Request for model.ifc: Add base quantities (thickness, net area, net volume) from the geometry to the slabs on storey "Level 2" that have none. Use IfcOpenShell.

First a look at what the model holds.

```python
import ifcopenshell
import ifcopenshell.util.element
import ifcopenshell.util.unit

model = ifcopenshell.open("model.ifc")
print(model.schema)
for unit_type in ("LENGTHUNIT", "AREAUNIT", "VOLUMEUNIT"):
    print(unit_type, ifcopenshell.util.unit.calculate_unit_scale(model, unit_type))
storey = next(s for s in model.by_type("IfcBuildingStorey") if s.Name == "Level 2")
slabs = [e for e in ifcopenshell.util.element.get_decomposition(storey) if e.is_a("IfcSlab")]
for e in sorted(slabs, key=lambda e: e.id()):
    print(e.id(), e.is_a(), e.Name, list(ifcopenshell.util.element.get_psets(e, qtos_only=True)), sep=" | ")
```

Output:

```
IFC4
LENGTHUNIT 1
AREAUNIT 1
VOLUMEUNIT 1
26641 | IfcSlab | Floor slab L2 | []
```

```python
import ifcopenshell
import ifcopenshell.api.pset
import ifcopenshell.geom
import ifcopenshell.util.element
import ifcopenshell.util.shape
import ifcopenshell.util.unit

model = ifcopenshell.open("model.ifc")
unit_scale = ifcopenshell.util.unit.calculate_unit_scale(model)
area_scale = ifcopenshell.util.unit.calculate_unit_scale(model, "AREAUNIT")
volume_scale = ifcopenshell.util.unit.calculate_unit_scale(model, "VOLUMEUNIT")
settings = ifcopenshell.geom.settings()

storey = next(s for s in model.by_type("IfcBuildingStorey") if s.Name == "Level 2")
slabs = [e for e in ifcopenshell.util.element.get_decomposition(storey) if e.is_a("IfcSlab")]

for e in sorted(slabs, key=lambda e: e.id()):
    if ifcopenshell.util.element.get_psets(e, qtos_only=True, should_inherit=False):
        continue
    # Geometry comes back in metres, in the element's own axes.
    shape = ifcopenshell.geom.create_shape(settings, e)
    values = {
        "Width": ifcopenshell.util.shape.get_z(shape.geometry) / unit_scale,
        "NetArea": ifcopenshell.util.shape.get_footprint_area(shape.geometry) / area_scale,
        "NetVolume": ifcopenshell.util.shape.get_volume(shape.geometry) / volume_scale,
    }
    qto = ifcopenshell.api.pset.add_qto(model, product=e, name="Qto_SlabBaseQuantities")
    ifcopenshell.api.pset.edit_qto(model, qto=qto, properties=values)
    print(e.id(), {k: round(v, 3) for k, v in values.items()})

model.write("model-out.ifc")
```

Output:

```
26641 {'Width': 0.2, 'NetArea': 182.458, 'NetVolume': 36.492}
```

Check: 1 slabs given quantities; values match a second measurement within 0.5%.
